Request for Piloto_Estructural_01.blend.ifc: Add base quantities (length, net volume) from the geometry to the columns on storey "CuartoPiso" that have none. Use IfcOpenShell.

First a look at what the model holds.

```python
import ifcopenshell
import ifcopenshell.util.element
import ifcopenshell.util.unit

model = ifcopenshell.open("Piloto_Estructural_01.blend.ifc")
print(model.schema)
for unit_type in ("LENGTHUNIT", "AREAUNIT", "VOLUMEUNIT"):
    print(unit_type, ifcopenshell.util.unit.calculate_unit_scale(model, unit_type))
storey = next(s for s in model.by_type("IfcBuildingStorey") if s.Name == "CuartoPiso")
columns = [e for e in ifcopenshell.util.element.get_decomposition(storey) if e.is_a("IfcColumn")]
for e in sorted(columns, key=lambda e: e.id()):
    print(e.id(), e.is_a(), e.Name, list(ifcopenshell.util.element.get_psets(e, qtos_only=True)), sep=" | ")
```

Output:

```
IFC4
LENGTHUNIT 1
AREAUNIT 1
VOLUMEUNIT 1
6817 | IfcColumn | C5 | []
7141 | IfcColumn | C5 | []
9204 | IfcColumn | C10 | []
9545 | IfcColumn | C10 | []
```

```python
import ifcopenshell
import ifcopenshell.api.pset
import ifcopenshell.geom
import ifcopenshell.util.element
import ifcopenshell.util.shape
import ifcopenshell.util.unit

model = ifcopenshell.open("Piloto_Estructural_01.blend.ifc")
unit_scale = ifcopenshell.util.unit.calculate_unit_scale(model)
volume_scale = ifcopenshell.util.unit.calculate_unit_scale(model, "VOLUMEUNIT")
settings = ifcopenshell.geom.settings()

storey = next(s for s in model.by_type("IfcBuildingStorey") if s.Name == "CuartoPiso")
columns = [e for e in ifcopenshell.util.element.get_decomposition(storey) if e.is_a("IfcColumn")]

for e in sorted(columns, key=lambda e: e.id()):
    if ifcopenshell.util.element.get_psets(e, qtos_only=True, should_inherit=False):
        continue
    # Geometry comes back in metres, in the element's own axes.
    shape = ifcopenshell.geom.create_shape(settings, e)
    values = {
        "Length": ifcopenshell.util.shape.get_z(shape.geometry) / unit_scale,
        "NetVolume": ifcopenshell.util.shape.get_volume(shape.geometry) / volume_scale,
    }
    qto = ifcopenshell.api.pset.add_qto(model, product=e, name="Qto_ColumnBaseQuantities")
    ifcopenshell.api.pset.edit_qto(model, qto=qto, properties=values)
    print(e.id(), {k: round(v, 3) for k, v in values.items()})

model.write("Piloto_Estructural_01.blend_rev.ifc")
```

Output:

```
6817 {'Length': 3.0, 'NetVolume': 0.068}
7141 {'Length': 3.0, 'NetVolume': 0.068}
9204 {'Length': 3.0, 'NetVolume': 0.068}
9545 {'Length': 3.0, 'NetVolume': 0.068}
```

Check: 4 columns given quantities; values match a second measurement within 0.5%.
